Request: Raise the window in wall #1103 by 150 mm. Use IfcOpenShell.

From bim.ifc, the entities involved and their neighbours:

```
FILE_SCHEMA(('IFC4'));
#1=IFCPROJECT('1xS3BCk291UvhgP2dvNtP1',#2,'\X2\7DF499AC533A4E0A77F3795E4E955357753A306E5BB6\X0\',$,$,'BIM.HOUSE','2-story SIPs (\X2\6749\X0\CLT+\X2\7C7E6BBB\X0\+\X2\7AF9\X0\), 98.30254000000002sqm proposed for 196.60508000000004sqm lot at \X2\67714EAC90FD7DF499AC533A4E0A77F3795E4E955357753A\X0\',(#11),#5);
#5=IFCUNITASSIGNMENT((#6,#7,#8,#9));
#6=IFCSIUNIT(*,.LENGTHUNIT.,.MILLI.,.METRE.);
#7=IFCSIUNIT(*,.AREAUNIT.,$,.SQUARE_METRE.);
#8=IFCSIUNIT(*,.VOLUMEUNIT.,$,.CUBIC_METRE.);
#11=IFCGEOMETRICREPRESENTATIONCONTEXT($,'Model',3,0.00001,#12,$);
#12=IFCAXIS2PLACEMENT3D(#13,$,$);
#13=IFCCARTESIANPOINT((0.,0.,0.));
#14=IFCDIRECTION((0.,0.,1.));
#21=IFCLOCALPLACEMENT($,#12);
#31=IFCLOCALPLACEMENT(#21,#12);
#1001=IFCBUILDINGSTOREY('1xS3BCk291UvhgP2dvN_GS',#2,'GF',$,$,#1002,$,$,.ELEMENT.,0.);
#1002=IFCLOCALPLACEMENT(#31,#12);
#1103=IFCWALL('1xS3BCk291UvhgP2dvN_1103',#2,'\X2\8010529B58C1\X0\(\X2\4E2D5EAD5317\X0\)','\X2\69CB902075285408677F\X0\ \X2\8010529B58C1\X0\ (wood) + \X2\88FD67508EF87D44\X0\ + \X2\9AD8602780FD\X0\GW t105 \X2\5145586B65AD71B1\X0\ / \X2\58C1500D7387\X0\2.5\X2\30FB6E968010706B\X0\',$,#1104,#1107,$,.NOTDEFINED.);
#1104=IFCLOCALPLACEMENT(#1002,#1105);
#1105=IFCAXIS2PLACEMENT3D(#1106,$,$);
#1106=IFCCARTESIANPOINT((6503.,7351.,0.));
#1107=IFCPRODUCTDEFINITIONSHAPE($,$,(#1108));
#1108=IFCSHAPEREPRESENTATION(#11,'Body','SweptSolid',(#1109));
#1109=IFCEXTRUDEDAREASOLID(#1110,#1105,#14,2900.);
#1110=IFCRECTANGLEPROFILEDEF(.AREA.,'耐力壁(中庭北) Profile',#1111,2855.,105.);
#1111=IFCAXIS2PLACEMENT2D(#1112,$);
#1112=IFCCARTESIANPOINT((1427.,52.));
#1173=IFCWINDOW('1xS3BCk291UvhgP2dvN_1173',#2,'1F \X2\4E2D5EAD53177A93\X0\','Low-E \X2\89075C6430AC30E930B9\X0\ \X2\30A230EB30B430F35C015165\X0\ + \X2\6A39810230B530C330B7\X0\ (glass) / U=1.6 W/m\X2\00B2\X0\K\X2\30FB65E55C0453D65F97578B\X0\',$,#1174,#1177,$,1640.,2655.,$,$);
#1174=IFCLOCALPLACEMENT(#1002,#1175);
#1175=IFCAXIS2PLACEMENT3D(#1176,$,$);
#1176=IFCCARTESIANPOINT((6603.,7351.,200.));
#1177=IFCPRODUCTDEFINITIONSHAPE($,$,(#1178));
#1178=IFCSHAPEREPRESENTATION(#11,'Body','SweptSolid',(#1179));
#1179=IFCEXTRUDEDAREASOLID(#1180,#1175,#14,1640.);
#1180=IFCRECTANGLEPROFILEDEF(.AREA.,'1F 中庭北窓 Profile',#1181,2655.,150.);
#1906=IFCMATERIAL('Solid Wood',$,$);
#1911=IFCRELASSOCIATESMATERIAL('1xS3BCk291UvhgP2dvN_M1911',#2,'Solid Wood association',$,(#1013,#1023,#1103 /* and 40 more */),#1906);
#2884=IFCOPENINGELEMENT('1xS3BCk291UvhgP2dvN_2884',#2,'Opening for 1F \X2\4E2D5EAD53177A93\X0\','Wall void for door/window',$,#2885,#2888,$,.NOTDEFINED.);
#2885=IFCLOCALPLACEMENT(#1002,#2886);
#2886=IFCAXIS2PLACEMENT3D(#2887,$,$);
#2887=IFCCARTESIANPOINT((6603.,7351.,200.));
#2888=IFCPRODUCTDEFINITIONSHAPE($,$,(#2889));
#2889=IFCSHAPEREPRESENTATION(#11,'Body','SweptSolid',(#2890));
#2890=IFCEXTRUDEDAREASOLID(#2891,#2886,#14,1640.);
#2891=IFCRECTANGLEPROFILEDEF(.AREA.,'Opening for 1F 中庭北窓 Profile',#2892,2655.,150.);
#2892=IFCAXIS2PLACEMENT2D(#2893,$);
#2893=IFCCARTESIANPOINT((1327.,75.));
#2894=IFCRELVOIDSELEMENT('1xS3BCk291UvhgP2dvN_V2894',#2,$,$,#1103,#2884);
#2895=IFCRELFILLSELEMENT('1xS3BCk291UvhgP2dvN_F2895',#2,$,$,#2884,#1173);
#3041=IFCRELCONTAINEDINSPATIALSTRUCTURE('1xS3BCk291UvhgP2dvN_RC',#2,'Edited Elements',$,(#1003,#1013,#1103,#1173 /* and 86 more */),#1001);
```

```python
import numpy as np
import ifcopenshell
import ifcopenshell.api.geometry
import ifcopenshell.util.placement
import ifcopenshell.util.unit

model = ifcopenshell.open("bim.ifc")
unit_scale = ifcopenshell.util.unit.calculate_unit_scale(model)

window = model.by_id(1173)
opening = window.FillsVoids[0].RelatingOpeningElement
dz = 150.0

shift = np.array([0.0, 0.0, dz])
# The window is not placed relative to its opening, so move both.
for product in (opening, window):
    matrix = ifcopenshell.util.placement.get_local_placement(product.ObjectPlacement)
    matrix[:3, 3] += shift
    ifcopenshell.api.geometry.edit_object_placement(model, product=product, matrix=matrix, is_si=False)

print(f"moved by {dz * unit_scale:+.3f} m")

model.write("bim_rev.ifc")
```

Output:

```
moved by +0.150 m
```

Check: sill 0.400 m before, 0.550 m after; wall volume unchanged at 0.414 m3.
